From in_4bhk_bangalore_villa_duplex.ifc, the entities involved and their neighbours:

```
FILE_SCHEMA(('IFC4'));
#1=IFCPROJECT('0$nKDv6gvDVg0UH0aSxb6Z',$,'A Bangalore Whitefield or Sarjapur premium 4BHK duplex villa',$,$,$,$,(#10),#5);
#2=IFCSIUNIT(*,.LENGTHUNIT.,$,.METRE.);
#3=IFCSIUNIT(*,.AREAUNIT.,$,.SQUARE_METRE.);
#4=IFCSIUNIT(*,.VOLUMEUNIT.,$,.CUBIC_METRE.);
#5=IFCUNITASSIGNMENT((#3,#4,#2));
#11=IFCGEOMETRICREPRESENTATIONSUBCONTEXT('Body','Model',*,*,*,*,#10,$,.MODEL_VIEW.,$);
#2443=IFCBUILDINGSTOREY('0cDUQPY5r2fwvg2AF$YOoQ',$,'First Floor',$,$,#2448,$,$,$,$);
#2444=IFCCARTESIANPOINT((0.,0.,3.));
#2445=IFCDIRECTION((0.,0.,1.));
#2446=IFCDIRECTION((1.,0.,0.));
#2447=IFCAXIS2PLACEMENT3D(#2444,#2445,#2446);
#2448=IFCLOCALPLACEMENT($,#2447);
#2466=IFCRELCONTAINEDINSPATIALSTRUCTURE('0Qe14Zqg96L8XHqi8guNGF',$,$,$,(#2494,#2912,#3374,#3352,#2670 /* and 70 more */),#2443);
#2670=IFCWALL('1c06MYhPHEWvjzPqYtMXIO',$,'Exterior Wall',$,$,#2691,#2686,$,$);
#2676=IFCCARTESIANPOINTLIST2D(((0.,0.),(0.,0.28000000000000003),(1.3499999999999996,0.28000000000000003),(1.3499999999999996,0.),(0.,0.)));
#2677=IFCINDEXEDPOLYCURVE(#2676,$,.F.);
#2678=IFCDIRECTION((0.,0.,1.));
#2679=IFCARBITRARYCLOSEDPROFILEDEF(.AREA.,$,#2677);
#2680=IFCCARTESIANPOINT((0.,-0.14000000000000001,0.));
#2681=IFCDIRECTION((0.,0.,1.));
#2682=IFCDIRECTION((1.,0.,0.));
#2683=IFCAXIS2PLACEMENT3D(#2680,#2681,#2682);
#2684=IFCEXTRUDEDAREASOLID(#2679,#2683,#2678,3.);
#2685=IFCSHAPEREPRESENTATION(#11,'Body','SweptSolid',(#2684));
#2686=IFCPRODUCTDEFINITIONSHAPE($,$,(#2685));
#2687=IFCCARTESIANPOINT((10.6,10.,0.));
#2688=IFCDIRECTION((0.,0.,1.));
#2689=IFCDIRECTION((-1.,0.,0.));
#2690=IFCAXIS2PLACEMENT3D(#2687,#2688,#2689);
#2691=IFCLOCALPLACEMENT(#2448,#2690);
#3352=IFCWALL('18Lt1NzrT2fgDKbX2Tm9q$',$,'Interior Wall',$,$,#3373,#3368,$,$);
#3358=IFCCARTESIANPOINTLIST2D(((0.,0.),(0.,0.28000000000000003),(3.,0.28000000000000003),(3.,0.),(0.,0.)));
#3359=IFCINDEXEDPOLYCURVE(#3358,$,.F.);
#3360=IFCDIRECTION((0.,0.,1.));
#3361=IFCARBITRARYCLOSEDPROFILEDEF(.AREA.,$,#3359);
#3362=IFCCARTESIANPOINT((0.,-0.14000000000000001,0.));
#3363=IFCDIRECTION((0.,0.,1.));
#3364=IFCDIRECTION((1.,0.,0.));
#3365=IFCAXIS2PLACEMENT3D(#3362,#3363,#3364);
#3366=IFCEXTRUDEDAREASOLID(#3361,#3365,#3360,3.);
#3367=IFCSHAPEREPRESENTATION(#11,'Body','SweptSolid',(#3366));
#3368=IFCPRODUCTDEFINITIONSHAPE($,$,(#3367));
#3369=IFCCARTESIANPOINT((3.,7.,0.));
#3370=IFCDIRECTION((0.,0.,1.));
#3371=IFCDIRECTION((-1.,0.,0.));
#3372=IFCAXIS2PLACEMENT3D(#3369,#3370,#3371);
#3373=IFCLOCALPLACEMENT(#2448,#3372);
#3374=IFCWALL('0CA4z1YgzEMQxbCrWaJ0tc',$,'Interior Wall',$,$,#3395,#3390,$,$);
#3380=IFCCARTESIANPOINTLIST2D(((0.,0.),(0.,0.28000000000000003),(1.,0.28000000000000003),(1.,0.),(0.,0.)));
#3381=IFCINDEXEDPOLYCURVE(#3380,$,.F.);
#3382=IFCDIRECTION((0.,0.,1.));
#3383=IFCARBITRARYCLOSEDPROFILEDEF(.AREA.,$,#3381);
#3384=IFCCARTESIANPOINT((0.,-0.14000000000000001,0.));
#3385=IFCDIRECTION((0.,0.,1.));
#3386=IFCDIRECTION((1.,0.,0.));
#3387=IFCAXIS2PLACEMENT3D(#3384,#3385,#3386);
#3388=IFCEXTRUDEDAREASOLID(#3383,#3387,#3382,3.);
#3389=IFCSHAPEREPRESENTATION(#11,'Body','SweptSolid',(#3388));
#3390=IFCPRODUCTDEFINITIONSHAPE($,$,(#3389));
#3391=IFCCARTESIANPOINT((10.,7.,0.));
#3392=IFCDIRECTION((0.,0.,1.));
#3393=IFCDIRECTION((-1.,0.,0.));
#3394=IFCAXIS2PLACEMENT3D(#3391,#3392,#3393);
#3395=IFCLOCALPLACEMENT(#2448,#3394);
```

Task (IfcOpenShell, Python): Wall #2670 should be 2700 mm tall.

```python
import ifcopenshell
import ifcopenshell.geom
import ifcopenshell.util.representation
import ifcopenshell.util.shape

model = ifcopenshell.open("in_4bhk_bangalore_villa_duplex.ifc")
settings = ifcopenshell.geom.settings()


def volume(element):
    """Net volume in cubic metres, openings subtracted."""
    shape = ifcopenshell.geom.create_shape(settings, element)
    return ifcopenshell.util.shape.get_volume(shape.geometry)


wall = model.by_guid("1c06MYhPHEWvjzPqYtMXIO")
before = volume(wall)

body = ifcopenshell.util.representation.get_representation(wall, "Model", "Body")
solid = body.Items[0]
old_height = solid.Depth
solid.Depth = 2.7
after = volume(wall)

print(f"height {old_height:g} -> {solid.Depth:g}, volume {before:.3f} -> {after:.3f} m3")

model.write("in_4bhk_bangalore_villa_duplex-out.ifc")
```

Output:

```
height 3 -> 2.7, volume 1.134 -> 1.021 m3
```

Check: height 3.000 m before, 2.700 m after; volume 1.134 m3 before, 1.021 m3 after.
